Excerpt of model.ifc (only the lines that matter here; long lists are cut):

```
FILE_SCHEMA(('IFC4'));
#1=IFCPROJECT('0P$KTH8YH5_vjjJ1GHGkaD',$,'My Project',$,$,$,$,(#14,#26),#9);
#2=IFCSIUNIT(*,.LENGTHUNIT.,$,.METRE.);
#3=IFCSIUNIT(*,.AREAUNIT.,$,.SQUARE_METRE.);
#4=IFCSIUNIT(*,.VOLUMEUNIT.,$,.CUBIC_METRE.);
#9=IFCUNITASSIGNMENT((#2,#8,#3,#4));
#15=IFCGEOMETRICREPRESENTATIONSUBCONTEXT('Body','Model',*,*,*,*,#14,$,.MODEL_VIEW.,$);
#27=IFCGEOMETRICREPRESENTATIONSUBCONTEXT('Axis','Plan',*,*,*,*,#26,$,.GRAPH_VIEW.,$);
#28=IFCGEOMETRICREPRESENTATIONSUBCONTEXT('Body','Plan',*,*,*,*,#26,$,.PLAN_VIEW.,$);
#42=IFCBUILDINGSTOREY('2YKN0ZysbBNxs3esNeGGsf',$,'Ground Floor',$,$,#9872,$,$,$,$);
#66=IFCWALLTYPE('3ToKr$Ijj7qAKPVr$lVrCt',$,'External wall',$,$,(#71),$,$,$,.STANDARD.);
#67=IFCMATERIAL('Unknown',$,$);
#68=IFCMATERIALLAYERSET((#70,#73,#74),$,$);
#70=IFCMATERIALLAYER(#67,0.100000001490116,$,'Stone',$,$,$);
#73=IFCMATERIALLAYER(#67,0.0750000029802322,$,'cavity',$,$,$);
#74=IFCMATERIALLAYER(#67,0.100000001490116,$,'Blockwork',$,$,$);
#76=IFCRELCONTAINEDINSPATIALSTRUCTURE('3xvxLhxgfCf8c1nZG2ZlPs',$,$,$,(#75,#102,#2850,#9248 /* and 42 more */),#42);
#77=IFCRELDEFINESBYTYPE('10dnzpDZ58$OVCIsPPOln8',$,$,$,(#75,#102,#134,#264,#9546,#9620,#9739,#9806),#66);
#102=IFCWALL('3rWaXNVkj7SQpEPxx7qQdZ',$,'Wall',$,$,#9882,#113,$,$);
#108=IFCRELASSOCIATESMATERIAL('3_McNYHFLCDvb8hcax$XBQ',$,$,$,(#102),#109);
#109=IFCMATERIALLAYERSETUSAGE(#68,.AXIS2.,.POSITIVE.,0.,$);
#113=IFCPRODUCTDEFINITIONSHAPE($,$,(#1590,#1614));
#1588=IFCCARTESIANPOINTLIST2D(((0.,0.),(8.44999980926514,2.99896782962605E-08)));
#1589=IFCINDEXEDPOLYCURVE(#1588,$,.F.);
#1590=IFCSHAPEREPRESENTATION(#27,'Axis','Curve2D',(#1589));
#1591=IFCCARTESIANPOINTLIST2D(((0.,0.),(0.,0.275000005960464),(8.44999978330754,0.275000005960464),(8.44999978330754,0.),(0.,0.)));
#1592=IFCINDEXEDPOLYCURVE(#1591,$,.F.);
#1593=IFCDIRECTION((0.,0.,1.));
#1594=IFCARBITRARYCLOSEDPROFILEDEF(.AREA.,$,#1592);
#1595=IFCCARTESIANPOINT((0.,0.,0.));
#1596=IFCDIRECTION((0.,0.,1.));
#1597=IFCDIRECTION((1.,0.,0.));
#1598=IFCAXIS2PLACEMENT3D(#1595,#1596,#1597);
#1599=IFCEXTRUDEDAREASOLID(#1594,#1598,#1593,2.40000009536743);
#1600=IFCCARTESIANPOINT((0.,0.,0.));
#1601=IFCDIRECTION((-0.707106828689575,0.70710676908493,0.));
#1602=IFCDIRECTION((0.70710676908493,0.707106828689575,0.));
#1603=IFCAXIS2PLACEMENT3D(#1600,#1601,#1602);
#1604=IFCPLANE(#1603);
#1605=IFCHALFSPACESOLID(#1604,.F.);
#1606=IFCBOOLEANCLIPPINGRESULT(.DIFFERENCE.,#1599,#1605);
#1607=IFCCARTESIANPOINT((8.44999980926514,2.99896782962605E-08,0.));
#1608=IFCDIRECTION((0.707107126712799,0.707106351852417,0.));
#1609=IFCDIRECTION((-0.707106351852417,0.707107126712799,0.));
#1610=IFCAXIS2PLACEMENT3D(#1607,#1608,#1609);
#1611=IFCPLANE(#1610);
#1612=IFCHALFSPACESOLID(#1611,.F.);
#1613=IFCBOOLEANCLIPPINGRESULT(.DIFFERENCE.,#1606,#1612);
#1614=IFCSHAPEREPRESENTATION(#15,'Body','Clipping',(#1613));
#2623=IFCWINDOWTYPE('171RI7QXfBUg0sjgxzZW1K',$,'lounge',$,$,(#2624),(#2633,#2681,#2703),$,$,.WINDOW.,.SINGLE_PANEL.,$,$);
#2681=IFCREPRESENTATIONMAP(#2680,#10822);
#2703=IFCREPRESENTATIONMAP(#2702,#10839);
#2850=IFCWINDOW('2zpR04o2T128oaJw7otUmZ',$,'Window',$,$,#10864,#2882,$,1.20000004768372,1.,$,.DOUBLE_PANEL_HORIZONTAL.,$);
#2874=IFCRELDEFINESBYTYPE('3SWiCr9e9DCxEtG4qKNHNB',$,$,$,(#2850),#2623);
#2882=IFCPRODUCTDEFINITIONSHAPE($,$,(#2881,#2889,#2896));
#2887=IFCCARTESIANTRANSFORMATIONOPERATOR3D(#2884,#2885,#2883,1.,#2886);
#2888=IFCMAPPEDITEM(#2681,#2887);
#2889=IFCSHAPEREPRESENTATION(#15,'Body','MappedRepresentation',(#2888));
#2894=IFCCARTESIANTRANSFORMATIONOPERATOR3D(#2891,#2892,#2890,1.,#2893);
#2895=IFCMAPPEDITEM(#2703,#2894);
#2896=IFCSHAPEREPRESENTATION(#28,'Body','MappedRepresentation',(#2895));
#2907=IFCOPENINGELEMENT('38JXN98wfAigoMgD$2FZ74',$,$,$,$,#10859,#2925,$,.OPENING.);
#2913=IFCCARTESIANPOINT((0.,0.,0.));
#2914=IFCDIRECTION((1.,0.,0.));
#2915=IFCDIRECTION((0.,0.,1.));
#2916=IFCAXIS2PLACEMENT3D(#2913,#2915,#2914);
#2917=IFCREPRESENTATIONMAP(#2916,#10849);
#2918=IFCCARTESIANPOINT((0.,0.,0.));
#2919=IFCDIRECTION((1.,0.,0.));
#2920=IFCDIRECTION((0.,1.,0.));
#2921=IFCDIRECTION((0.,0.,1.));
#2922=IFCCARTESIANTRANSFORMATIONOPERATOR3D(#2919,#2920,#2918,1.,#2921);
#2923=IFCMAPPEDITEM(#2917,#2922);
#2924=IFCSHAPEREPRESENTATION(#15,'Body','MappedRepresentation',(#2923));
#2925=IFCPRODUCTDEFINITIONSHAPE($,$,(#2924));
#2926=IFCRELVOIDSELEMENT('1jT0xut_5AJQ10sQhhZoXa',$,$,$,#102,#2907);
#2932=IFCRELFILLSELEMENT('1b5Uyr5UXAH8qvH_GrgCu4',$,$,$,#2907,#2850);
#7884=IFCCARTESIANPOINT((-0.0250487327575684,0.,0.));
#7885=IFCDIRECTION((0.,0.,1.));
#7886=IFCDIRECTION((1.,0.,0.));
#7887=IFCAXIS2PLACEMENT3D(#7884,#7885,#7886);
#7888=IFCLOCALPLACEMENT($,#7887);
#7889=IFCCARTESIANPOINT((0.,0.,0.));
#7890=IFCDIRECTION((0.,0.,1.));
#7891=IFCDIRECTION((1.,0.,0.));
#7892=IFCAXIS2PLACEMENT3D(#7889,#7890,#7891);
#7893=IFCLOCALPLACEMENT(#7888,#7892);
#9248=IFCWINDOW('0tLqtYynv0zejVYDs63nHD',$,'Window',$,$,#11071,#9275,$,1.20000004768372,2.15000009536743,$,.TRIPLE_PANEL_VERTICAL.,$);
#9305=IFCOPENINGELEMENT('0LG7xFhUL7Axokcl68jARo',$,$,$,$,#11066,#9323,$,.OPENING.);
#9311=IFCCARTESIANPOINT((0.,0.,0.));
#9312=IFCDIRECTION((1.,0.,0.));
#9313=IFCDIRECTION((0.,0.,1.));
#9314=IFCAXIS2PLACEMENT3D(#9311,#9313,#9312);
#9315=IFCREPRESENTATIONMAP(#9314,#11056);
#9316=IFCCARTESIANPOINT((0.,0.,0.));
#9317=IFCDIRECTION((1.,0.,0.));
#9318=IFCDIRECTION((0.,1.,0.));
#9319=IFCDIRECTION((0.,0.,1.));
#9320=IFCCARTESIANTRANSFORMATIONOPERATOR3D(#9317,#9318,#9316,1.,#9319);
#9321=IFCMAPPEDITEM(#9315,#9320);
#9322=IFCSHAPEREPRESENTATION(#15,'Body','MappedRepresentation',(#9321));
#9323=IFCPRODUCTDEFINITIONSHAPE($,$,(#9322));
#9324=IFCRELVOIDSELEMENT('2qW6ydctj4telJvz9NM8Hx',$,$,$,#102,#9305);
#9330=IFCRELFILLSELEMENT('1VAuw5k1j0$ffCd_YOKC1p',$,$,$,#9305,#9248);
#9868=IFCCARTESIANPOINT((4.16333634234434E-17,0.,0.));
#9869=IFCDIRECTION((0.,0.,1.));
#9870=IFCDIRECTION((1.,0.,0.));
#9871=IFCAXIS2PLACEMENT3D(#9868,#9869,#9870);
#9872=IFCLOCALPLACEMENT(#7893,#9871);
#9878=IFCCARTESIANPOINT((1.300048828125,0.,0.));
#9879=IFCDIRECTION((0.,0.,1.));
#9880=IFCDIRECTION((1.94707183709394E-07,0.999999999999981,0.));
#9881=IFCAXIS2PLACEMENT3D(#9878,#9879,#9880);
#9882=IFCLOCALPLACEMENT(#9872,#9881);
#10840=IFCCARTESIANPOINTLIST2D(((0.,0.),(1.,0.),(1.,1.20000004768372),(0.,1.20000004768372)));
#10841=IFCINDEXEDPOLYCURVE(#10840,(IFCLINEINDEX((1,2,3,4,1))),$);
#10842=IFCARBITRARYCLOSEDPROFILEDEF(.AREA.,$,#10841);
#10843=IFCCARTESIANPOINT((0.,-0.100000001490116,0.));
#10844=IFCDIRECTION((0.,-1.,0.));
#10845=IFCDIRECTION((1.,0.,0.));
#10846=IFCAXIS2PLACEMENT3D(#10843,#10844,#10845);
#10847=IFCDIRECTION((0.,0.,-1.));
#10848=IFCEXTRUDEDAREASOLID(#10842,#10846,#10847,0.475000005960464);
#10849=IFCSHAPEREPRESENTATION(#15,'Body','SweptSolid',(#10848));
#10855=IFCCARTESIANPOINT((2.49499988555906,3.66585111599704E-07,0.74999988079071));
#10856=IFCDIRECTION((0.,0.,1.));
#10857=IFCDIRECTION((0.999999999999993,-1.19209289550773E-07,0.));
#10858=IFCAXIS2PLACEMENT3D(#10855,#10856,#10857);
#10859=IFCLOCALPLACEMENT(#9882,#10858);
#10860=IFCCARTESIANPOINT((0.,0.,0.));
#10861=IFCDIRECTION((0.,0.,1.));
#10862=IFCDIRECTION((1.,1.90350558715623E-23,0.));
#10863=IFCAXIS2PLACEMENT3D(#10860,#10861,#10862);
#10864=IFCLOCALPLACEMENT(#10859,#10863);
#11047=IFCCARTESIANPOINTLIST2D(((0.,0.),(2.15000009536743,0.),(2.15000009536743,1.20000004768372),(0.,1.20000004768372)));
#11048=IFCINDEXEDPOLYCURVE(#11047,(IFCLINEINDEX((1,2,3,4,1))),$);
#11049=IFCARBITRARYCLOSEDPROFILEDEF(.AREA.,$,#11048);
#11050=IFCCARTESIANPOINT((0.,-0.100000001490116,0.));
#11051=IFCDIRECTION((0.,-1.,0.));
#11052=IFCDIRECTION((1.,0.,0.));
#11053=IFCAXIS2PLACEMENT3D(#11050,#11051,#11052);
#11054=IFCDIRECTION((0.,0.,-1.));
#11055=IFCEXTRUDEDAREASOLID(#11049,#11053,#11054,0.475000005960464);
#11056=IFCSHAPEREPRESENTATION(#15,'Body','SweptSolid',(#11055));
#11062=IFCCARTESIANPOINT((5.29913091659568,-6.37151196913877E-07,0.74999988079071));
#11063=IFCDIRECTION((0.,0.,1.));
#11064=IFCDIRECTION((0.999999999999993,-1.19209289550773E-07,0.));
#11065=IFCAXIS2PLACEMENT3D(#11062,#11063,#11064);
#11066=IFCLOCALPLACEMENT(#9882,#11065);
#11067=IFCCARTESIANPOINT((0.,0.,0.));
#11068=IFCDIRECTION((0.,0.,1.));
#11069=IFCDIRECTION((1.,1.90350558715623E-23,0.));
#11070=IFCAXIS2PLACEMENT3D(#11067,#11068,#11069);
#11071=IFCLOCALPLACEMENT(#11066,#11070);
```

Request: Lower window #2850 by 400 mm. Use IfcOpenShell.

```python
import numpy as np
import ifcopenshell
import ifcopenshell.api.geometry
import ifcopenshell.util.placement
import ifcopenshell.util.unit

model = ifcopenshell.open("model.ifc")
unit_scale = ifcopenshell.util.unit.calculate_unit_scale(model)

window = model.by_guid("2zpR04o2T128oaJw7otUmZ")
opening = window.FillsVoids[0].RelatingOpeningElement
dz = -0.4

shift = np.array([0.0, 0.0, dz])
# The window is placed relative to its opening, so it follows when the opening moves.
matrix = ifcopenshell.util.placement.get_local_placement(opening.ObjectPlacement)
matrix[:3, 3] += shift
ifcopenshell.api.geometry.edit_object_placement(
    model, product=opening, matrix=matrix, is_si=False, should_transform_children=True
)

print(f"moved by {dz * unit_scale:+.3f} m")

model.write("model-out.ifc")
```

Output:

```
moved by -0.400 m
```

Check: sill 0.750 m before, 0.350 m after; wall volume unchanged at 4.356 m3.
